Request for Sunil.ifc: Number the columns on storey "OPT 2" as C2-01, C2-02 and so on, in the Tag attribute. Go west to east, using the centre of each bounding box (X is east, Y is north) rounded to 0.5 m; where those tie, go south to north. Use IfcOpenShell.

First a look at what the model holds.

```python
import ifcopenshell
import ifcopenshell.util.element
import ifcopenshell.util.placement

model = ifcopenshell.open("Sunil.ifc")
print(model.schema)
storey = next(s for s in model.by_type("IfcBuildingStorey") if s.Name == "OPT 2")
columns = [e for e in ifcopenshell.util.element.get_decomposition(storey) if e.is_a("IfcColumn")]
for e in sorted(columns, key=lambda e: e.id()):
    origin = ifcopenshell.util.placement.get_local_placement(e.ObjectPlacement)[:3, 3]
    print(e.id(), e.Tag, e.Name, origin.round(2) + 0.0, sep=" | ")
```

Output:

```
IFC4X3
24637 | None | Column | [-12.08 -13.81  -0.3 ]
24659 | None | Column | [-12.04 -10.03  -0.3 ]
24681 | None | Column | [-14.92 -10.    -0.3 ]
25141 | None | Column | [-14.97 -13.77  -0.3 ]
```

```python
import ifcopenshell
import ifcopenshell.geom
import ifcopenshell.util.element
import ifcopenshell.util.shape

model = ifcopenshell.open("Sunil.ifc")
settings = ifcopenshell.geom.settings()
settings.set("use-world-coords", True)


def centre(element):
    shape = ifcopenshell.geom.create_shape(settings, element)
    return ifcopenshell.util.shape.get_bbox_centroid(shape.geometry)


storey = next(s for s in model.by_type("IfcBuildingStorey") if s.Name == "OPT 2")
columns = [e for e in ifcopenshell.util.element.get_decomposition(storey) if e.is_a("IfcColumn")]

# Insertion points can sit at a corner or the storey origin, so sort by the geometry (in metres).
centres = {e: centre(e) for e in columns}
columns.sort(key=lambda e: (round(centres[e][0] / 0.5), centres[e][1]))

for i, e in enumerate(columns, start=1):
    number = f"C2-{i:02d}"
    e.Tag = number
    print(e.id(), number)

model.write("Sunil_rev.ifc")
```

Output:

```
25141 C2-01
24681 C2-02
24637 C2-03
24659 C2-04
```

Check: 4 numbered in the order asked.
